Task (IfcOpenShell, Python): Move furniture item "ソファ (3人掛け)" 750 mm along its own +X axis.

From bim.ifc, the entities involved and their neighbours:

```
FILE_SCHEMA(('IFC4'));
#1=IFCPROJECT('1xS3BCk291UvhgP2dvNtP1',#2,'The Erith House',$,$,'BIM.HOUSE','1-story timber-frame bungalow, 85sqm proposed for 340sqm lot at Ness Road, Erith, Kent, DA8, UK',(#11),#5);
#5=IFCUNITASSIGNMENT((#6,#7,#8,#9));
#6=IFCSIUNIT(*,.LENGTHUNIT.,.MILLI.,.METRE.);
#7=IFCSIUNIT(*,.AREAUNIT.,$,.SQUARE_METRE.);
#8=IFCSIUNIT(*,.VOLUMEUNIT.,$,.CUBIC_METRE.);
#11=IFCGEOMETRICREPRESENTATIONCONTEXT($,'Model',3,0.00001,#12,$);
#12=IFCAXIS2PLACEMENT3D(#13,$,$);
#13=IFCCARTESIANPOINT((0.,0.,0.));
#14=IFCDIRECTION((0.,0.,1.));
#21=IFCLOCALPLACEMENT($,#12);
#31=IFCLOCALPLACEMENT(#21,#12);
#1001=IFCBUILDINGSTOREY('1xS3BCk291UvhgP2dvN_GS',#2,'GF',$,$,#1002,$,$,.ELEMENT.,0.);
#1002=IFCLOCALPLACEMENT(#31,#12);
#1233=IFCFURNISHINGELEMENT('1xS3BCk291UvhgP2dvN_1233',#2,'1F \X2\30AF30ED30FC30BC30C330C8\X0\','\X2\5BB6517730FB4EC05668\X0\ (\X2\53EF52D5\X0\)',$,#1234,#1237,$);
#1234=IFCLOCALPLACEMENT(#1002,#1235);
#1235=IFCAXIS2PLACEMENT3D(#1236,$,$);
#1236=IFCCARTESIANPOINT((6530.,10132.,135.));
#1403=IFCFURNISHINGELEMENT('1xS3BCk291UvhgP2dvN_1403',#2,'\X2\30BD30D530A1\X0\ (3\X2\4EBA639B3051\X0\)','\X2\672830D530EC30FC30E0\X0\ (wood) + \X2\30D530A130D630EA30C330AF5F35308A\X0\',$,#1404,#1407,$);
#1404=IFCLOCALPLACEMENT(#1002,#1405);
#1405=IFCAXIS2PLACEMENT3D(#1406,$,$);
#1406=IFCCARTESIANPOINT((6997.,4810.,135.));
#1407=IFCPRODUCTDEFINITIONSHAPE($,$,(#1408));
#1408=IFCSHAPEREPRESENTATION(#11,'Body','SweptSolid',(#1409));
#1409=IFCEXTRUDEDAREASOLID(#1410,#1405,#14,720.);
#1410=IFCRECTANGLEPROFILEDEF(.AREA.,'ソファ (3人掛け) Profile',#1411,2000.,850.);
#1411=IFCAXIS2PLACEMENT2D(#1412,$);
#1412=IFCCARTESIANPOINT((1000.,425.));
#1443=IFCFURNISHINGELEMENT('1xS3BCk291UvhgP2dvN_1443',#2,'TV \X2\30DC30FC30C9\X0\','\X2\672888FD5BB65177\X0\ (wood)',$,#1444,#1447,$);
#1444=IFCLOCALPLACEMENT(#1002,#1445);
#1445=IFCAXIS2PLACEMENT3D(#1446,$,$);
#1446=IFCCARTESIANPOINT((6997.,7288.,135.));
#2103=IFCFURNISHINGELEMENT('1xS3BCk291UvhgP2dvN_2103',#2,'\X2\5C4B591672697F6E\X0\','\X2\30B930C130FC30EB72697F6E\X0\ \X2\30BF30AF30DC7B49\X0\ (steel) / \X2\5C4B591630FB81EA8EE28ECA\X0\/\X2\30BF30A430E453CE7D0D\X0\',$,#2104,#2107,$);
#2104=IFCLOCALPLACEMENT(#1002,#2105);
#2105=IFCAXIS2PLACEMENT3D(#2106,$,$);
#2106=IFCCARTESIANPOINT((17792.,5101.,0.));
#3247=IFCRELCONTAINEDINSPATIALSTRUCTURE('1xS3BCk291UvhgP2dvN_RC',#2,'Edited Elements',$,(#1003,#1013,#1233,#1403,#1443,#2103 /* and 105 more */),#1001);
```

```python
import ifcopenshell
import ifcopenshell.api.geometry
import ifcopenshell.util.placement

model = ifcopenshell.open("bim.ifc")

item = model.by_guid("1xS3BCk291UvhgP2dvN_1403")
matrix = ifcopenshell.util.placement.get_local_placement(item.ObjectPlacement)
matrix[:3, 3] += matrix[:3, 0] * 750.0
ifcopenshell.api.geometry.edit_object_placement(model, product=item, matrix=matrix, is_si=False)

print(ifcopenshell.util.placement.get_local_placement(item.ObjectPlacement).round(3) + 0.0)

model.write("bim_rev.ifc")
```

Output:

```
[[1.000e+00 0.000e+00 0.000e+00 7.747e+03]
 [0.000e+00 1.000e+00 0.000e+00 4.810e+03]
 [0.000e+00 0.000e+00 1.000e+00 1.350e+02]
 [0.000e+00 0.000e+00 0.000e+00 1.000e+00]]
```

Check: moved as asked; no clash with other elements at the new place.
